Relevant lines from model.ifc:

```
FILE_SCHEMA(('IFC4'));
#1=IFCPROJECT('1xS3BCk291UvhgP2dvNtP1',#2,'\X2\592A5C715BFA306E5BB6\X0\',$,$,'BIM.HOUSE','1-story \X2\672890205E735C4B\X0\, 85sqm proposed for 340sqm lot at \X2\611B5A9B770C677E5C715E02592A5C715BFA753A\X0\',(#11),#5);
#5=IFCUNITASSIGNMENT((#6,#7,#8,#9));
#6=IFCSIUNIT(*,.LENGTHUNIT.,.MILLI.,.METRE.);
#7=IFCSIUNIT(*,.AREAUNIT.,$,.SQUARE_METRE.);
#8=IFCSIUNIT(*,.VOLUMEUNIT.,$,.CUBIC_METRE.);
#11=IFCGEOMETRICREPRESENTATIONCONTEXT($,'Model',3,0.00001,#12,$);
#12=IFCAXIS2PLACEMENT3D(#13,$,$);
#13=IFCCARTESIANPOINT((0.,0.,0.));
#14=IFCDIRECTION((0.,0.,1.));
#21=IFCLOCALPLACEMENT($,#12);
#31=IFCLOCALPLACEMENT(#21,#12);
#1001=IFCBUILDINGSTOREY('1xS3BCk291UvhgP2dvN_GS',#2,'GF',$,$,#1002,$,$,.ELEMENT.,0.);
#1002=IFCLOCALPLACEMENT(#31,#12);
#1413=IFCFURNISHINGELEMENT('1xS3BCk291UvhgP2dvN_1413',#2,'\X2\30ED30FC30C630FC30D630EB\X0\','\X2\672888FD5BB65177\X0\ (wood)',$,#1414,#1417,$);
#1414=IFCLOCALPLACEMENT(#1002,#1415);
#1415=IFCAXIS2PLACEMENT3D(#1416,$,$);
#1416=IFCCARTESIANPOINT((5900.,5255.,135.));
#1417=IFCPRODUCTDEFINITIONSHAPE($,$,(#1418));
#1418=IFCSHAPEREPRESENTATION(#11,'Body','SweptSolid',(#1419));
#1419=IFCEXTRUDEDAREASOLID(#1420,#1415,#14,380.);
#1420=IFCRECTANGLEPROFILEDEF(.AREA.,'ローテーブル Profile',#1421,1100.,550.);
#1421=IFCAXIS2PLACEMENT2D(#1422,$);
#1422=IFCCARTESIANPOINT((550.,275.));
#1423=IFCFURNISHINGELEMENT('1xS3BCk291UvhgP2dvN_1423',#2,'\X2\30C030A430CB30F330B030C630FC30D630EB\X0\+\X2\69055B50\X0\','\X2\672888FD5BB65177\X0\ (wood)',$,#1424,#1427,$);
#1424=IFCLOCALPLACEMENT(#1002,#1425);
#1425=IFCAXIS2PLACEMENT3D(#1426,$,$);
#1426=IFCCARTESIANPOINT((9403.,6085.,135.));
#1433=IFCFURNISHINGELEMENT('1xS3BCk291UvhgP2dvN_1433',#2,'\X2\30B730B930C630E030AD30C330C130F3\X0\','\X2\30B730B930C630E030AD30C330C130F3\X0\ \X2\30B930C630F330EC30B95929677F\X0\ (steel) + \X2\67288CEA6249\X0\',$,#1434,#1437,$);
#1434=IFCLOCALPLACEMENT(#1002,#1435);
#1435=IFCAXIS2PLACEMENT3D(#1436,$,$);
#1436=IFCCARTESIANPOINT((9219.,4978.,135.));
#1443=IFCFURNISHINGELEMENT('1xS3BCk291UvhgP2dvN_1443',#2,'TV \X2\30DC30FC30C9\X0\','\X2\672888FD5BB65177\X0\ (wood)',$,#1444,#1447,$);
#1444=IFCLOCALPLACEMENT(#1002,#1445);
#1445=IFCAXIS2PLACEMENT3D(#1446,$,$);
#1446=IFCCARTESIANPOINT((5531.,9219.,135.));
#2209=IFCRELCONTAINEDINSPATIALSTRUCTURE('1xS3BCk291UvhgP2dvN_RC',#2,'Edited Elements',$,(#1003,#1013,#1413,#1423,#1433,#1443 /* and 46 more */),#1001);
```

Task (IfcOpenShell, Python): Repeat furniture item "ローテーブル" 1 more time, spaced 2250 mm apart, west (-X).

```python
import numpy as np
import ifcopenshell
import ifcopenshell.api.geometry
import ifcopenshell.api.root
import ifcopenshell.util.element
import ifcopenshell.util.placement
import ifcopenshell.util.unit

model = ifcopenshell.open("model.ifc")
unit_scale = ifcopenshell.util.unit.calculate_unit_scale(model)


def reuse_history(source, copy):
    """copy_class also copies each property set's owner history, people and application; keep the originals."""
    for rel in copy.IsDefinedBy:
        if rel.is_a("IfcRelDefinesByProperties") and (history := rel.RelatingPropertyDefinition.OwnerHistory):
            rel.RelatingPropertyDefinition.OwnerHistory = source.OwnerHistory
            ifcopenshell.util.element.remove_deep2(model, history)


source = model.by_guid("1xS3BCk291UvhgP2dvN_1413")
base = ifcopenshell.util.placement.get_local_placement(source.ObjectPlacement)
step = np.array([-1.0, 0.0, 0.0]) * 2.25 / unit_scale

for i in range(1, 2):
    copy = ifcopenshell.api.root.copy_class(model, product=source)
    copy.Representation = ifcopenshell.util.element.copy_deep(
        model, source.Representation, exclude=["IfcGeometricRepresentationContext", "IfcRepresentationMap"]
    )
    reuse_history(source, copy)
    matrix = base.copy()
    matrix[:3, 3] += i * step
    print("added at", matrix[:3, 3].round(3) + 0.0)
    ifcopenshell.api.geometry.edit_object_placement(model, product=copy, matrix=matrix, is_si=False)

model.write("model_edited.ifc")
```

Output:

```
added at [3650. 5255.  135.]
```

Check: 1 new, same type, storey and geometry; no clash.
